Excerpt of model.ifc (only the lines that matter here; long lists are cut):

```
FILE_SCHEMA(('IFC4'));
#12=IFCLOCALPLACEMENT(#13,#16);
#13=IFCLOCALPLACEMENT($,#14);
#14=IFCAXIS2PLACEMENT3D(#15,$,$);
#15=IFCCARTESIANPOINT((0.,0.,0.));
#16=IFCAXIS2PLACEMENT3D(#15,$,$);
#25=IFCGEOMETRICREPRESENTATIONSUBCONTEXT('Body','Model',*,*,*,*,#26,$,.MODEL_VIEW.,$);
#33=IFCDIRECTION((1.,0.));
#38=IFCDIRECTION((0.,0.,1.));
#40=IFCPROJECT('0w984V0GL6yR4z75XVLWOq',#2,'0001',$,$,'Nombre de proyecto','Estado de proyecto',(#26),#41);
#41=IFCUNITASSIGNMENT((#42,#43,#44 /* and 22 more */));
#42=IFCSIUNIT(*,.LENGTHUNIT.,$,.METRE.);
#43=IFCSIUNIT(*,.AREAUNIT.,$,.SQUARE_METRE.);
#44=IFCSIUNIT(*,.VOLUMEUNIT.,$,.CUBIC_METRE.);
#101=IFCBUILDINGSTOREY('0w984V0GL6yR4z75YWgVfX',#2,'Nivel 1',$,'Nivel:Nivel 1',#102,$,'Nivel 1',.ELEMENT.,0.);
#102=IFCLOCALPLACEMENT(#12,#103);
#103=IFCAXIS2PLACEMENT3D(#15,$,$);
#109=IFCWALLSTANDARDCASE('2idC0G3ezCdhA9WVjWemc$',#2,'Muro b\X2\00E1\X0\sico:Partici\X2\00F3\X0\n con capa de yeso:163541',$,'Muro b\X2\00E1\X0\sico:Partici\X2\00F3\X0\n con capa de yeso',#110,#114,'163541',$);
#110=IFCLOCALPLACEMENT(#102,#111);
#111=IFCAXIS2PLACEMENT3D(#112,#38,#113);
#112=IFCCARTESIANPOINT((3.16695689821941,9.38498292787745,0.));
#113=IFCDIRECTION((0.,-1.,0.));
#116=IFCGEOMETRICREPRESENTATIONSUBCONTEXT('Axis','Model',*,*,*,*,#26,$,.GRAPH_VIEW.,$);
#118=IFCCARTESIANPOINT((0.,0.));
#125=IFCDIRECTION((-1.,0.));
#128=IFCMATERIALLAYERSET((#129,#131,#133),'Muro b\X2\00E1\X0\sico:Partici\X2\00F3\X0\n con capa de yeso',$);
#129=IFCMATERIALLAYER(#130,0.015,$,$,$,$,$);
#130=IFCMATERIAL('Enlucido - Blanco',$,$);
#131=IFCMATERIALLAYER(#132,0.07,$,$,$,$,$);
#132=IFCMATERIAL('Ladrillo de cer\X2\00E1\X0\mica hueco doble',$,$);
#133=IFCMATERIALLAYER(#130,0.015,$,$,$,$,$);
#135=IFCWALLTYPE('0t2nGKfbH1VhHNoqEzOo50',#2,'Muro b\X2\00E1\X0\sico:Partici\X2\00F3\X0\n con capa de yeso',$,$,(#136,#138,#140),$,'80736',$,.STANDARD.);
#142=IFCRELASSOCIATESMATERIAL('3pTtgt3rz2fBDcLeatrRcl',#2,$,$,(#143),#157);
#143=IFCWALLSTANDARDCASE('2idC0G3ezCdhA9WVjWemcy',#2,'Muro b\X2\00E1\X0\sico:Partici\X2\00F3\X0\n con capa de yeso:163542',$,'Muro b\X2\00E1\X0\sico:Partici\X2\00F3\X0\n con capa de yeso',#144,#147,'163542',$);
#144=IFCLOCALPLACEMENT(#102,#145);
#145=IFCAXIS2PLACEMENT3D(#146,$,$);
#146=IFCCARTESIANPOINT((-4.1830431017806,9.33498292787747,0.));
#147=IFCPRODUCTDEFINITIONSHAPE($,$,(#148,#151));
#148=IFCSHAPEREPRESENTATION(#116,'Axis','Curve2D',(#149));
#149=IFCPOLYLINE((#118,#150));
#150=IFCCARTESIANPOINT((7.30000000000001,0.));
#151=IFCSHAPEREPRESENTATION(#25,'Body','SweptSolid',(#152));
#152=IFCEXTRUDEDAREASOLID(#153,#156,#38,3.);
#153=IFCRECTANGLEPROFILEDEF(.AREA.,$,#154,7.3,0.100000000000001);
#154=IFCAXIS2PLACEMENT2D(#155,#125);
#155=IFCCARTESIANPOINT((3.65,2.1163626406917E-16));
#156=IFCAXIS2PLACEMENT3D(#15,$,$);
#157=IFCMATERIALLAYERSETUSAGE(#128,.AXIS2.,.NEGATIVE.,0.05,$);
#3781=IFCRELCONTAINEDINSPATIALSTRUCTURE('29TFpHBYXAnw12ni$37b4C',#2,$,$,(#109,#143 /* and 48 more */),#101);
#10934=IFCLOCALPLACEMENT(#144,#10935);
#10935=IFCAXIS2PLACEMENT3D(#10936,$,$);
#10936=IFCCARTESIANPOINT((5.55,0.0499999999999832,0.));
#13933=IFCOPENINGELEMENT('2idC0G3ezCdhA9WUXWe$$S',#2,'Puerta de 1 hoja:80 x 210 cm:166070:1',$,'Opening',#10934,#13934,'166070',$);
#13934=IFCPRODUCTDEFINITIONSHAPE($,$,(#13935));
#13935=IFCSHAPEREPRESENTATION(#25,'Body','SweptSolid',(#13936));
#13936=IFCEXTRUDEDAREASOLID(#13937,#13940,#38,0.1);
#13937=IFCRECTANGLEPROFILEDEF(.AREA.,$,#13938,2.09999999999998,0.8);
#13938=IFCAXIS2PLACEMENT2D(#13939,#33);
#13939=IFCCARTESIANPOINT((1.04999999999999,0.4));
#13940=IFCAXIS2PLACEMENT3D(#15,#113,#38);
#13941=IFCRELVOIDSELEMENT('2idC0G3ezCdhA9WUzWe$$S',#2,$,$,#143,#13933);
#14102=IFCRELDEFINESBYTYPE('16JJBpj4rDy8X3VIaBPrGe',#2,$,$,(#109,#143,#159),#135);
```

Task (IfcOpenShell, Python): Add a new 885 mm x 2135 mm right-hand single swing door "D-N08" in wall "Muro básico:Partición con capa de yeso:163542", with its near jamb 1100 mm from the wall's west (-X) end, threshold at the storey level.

```python
import numpy as np
import ifcopenshell
import ifcopenshell.api.feature
import ifcopenshell.api.geometry
import ifcopenshell.api.root
import ifcopenshell.api.spatial
import ifcopenshell.geom
import ifcopenshell.util.element
import ifcopenshell.util.placement
import ifcopenshell.util.representation
import ifcopenshell.util.shape
import ifcopenshell.util.unit

model = ifcopenshell.open("model.ifc")
unit_scale = ifcopenshell.util.unit.calculate_unit_scale(model)
settings = ifcopenshell.geom.settings()


def volume(element):
    """Net volume in cubic metres, openings subtracted."""
    shape = ifcopenshell.geom.create_shape(settings, element)
    return ifcopenshell.util.shape.get_volume(shape.geometry)


wall = model.by_guid("2idC0G3ezCdhA9WVjWemcy")
storey = ifcopenshell.util.element.get_container(wall, ifc_class="IfcBuildingStorey")
context = ifcopenshell.util.representation.get_context(model, "Model", "Body", "MODEL_VIEW")
before = volume(wall)

width, height, from_end, sill = 0.885, 2.135, 1.1, 0.0  # metres

# The wall runs along its own X axis, and the end named is its -X end.
wall_shape = ifcopenshell.geom.create_shape(settings, wall)
x, y, z = ifcopenshell.util.shape.get_vertices(wall_shape.geometry).T
start = x.min() + from_end
face, thickness = float(y.min()), float(y.max() - y.min())
wall_matrix = ifcopenshell.util.placement.get_local_placement(wall.ObjectPlacement)
level = ifcopenshell.util.placement.get_local_placement(storey.ObjectPlacement)[2, 3]


def in_wall(x, y):
    """Placement at x, y metres in the wall's axes, at sill height."""
    matrix = wall_matrix.copy()
    matrix[:, 3] = wall_matrix @ np.array([x / unit_scale, y / unit_scale, 0.0, 1.0])
    matrix[2, 3] = level + sill / unit_scale
    return matrix


# Opening: a box that overshoots both wall faces by 50 mm.
opening = ifcopenshell.api.root.create_entity(model, ifc_class="IfcOpeningElement", predefined_type="OPENING")
box = ifcopenshell.api.geometry.add_wall_representation(
    model, context=context, length=width, height=height, thickness=thickness + 0.1
)
ifcopenshell.api.geometry.assign_representation(model, product=opening, representation=box)
ifcopenshell.api.geometry.edit_object_placement(model, product=opening, matrix=in_wall(start, face - 0.05), is_si=False)
ifcopenshell.api.feature.add_feature(model, feature=opening, element=wall)

door = ifcopenshell.api.root.create_entity(model, ifc_class="IfcDoor", name="D-N08", predefined_type="DOOR")
door.OverallWidth, door.OverallHeight = width / unit_scale, height / unit_scale
door.OperationType = "SINGLE_SWING_RIGHT"
body = ifcopenshell.api.geometry.add_door_representation(
    model,
    context=context,
    overall_width=door.OverallWidth,
    overall_height=door.OverallHeight,
    operation_type="SINGLE_SWING_RIGHT",
    lining_properties={"LiningDepth": thickness / unit_scale, "ThresholdDepth": thickness / unit_scale},
)
ifcopenshell.api.geometry.assign_representation(model, product=door, representation=body)
ifcopenshell.api.spatial.assign_container(model, products=[door], relating_structure=storey)
ifcopenshell.api.feature.add_filling(model, opening=opening, element=door)

# The lining spans the wall, so the door starts at the wall face.
ifcopenshell.api.geometry.edit_object_placement(model, product=door, matrix=in_wall(start, face), is_si=False)

after = volume(wall)

print(f"wall volume {before:.3f} -> {after:.3f} m3")

model.write("model_updated.ifc")
```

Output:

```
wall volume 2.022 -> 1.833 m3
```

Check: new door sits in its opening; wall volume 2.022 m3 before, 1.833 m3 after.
